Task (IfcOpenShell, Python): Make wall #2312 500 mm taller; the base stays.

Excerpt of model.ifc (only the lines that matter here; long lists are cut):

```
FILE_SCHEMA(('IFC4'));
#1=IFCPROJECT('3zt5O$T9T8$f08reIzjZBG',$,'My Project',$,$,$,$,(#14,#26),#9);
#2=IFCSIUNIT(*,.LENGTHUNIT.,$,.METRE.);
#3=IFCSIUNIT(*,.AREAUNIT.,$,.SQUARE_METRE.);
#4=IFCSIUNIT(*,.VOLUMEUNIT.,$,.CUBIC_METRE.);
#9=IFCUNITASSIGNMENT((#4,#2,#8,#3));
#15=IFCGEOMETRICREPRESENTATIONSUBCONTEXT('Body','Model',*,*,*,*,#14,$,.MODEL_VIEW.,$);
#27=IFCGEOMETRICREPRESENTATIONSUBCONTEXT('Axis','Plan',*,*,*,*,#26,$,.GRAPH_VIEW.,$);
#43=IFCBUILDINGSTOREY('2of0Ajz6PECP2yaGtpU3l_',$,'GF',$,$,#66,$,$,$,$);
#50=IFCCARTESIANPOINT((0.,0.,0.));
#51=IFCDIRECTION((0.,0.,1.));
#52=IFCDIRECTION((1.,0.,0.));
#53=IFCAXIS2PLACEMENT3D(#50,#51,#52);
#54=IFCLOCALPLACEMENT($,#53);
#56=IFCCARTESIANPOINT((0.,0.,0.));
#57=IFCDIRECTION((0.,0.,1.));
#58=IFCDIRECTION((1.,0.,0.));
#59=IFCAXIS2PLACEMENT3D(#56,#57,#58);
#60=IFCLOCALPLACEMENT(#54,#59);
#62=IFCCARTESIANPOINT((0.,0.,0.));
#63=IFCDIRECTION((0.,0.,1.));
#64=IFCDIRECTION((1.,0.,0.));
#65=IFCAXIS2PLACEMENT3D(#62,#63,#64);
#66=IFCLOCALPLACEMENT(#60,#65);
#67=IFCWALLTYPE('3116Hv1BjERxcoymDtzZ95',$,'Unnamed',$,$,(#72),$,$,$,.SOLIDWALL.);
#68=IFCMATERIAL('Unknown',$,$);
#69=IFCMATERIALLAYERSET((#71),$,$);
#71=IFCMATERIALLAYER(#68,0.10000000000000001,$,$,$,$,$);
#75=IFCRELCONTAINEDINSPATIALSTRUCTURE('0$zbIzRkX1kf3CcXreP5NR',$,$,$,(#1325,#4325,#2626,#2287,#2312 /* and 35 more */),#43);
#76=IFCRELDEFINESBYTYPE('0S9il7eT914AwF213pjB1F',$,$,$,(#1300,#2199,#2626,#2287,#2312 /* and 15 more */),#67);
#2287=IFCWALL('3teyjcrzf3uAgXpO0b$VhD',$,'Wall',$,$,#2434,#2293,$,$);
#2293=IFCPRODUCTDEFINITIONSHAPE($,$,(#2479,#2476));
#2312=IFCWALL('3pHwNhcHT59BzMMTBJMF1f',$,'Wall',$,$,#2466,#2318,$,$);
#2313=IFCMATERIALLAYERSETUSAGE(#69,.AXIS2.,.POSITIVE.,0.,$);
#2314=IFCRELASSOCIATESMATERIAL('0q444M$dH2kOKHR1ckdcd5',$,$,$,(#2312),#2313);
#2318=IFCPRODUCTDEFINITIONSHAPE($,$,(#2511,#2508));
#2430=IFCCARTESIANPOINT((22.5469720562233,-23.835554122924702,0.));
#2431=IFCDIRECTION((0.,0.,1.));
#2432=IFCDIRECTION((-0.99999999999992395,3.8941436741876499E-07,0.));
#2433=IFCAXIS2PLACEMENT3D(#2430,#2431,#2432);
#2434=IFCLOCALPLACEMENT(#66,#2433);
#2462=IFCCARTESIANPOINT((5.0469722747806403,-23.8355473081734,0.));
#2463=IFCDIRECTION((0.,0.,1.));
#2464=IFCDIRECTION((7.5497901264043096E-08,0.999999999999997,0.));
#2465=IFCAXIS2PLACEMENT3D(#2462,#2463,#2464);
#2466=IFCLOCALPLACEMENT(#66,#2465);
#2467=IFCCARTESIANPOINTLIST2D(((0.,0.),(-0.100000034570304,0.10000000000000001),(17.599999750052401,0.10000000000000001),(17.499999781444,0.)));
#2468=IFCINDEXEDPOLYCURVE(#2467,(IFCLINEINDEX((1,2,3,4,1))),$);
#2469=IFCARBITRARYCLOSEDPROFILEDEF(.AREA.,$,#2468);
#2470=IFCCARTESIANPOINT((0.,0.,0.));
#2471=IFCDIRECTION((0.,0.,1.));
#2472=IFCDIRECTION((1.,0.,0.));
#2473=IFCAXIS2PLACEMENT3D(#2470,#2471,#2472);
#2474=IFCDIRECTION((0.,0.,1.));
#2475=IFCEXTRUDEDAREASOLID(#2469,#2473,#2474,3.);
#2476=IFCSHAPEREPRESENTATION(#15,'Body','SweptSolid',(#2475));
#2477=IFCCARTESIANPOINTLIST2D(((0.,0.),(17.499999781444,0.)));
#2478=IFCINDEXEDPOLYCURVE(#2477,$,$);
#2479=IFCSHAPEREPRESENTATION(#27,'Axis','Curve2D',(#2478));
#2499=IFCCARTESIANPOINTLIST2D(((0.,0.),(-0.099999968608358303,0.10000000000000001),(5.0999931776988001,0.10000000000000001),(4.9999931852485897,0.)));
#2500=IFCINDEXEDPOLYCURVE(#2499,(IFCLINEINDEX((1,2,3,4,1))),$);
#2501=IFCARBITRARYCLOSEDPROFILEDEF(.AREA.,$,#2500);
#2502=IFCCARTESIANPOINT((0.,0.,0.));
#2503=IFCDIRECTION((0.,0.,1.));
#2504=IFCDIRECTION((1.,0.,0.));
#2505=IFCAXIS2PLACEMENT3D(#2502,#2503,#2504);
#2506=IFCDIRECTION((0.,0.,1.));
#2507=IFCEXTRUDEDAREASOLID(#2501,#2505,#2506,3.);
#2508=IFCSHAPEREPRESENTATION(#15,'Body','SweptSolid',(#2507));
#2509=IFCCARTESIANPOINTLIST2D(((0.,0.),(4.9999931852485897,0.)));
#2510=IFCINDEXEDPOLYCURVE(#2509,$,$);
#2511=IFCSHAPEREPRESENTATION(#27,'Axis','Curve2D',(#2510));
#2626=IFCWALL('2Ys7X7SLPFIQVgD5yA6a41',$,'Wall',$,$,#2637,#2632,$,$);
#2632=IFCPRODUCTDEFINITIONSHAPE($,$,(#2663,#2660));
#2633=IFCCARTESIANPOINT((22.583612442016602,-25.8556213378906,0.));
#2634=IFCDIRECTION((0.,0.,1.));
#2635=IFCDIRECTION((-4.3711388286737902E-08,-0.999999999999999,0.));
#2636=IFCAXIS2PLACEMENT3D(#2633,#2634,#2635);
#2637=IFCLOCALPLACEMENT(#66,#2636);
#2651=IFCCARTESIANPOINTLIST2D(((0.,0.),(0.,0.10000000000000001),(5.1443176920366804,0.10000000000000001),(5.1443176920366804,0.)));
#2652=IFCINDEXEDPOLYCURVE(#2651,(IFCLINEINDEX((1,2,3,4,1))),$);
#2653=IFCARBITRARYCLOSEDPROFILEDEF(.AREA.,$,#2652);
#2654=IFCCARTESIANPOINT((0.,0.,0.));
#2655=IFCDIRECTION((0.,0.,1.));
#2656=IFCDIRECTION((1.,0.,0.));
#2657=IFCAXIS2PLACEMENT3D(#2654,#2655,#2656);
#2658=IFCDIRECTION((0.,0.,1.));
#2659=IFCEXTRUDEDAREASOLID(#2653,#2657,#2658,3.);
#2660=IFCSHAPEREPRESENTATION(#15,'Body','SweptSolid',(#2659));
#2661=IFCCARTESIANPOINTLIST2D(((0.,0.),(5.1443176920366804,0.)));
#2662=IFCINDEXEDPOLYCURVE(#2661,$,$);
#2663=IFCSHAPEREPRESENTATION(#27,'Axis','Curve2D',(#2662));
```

```python
import ifcopenshell
import ifcopenshell.geom
import ifcopenshell.util.representation
import ifcopenshell.util.shape

model = ifcopenshell.open("model.ifc")
settings = ifcopenshell.geom.settings()


def volume(element):
    """Net volume in cubic metres, openings subtracted."""
    shape = ifcopenshell.geom.create_shape(settings, element)
    return ifcopenshell.util.shape.get_volume(shape.geometry)


wall = model.by_guid("3pHwNhcHT59BzMMTBJMF1f")
before = volume(wall)

body = ifcopenshell.util.representation.get_representation(wall, "Model", "Body")
solid = body.Items[0]
old_height = solid.Depth
solid.Depth += 0.5
after = volume(wall)

print(f"height {old_height:g} -> {solid.Depth:g}, volume {before:.3f} -> {after:.3f} m3")

model.write("model-out.ifc")
```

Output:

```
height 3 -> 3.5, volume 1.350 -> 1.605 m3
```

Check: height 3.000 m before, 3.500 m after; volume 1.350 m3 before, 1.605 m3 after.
